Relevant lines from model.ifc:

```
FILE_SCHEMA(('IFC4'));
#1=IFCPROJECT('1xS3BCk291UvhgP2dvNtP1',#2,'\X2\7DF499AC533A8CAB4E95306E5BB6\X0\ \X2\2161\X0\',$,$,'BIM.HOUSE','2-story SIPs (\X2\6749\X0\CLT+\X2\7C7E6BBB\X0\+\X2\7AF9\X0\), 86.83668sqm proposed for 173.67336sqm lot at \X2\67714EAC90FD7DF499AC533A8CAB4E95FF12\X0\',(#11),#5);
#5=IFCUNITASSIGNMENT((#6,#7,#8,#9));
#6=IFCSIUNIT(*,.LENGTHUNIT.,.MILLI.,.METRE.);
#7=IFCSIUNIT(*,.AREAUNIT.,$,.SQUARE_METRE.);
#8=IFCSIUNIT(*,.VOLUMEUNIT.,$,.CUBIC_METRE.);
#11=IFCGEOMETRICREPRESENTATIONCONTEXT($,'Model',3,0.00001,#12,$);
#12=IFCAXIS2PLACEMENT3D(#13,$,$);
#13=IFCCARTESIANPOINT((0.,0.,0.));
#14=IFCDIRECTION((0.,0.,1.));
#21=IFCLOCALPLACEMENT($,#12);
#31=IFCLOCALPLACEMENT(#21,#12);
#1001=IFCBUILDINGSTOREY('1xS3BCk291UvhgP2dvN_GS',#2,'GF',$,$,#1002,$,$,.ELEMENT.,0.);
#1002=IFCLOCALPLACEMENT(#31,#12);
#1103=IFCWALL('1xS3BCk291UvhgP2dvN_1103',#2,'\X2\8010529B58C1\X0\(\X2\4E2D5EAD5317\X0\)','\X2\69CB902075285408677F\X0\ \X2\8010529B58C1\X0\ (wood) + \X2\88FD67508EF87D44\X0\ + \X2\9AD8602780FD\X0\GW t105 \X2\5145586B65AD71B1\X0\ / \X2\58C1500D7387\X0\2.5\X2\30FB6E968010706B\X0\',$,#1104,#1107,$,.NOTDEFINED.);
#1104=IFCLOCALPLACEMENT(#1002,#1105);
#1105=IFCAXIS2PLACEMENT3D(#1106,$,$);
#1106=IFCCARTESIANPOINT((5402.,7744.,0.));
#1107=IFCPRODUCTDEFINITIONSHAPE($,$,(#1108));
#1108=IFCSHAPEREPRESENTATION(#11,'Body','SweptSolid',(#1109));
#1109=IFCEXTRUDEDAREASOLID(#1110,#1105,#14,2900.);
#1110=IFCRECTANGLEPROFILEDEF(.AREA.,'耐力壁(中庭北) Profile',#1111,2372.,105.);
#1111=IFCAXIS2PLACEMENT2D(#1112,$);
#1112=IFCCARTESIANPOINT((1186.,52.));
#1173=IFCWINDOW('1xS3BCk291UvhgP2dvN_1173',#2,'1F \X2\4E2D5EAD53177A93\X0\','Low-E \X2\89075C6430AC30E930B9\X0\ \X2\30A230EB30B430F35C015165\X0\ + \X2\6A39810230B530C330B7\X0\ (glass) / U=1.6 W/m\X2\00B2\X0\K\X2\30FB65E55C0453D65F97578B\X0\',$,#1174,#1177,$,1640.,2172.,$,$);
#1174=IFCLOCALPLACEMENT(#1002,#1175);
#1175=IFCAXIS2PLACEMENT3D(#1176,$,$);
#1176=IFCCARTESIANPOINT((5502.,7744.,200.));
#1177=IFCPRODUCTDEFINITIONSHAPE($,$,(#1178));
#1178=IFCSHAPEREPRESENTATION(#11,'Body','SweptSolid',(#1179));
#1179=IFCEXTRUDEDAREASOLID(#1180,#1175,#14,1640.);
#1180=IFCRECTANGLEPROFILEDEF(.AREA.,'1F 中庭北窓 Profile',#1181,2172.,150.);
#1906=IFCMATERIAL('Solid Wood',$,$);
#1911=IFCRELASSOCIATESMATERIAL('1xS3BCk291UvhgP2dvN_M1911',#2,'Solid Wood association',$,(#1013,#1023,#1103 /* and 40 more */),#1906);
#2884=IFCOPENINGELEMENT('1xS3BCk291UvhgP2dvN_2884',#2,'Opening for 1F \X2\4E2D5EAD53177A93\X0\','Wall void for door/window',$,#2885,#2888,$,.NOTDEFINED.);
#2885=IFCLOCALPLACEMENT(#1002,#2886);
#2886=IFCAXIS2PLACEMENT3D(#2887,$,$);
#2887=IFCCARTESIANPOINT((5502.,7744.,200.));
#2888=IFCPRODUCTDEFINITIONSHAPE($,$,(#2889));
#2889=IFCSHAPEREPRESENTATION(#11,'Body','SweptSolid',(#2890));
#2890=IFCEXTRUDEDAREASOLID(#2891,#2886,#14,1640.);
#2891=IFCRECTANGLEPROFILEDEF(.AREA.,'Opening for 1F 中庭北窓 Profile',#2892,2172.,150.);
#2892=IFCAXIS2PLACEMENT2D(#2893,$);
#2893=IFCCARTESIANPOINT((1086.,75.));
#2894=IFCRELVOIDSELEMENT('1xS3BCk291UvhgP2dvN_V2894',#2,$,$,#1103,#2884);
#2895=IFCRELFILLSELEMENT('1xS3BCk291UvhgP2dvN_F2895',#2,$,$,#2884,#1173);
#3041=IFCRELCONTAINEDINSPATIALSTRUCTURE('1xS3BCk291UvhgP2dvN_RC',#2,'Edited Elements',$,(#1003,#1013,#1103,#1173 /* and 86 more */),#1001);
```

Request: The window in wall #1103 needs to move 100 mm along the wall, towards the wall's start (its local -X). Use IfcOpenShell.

```python
import ifcopenshell
import ifcopenshell.api.geometry
import ifcopenshell.util.placement

model = ifcopenshell.open("model.ifc")

window = model.by_guid("1xS3BCk291UvhgP2dvN_1173")
opening = window.FillsVoids[0].RelatingOpeningElement
wall = opening.VoidsElements[0].RelatingBuildingElement

wall_matrix = ifcopenshell.util.placement.get_local_placement(wall.ObjectPlacement)
shift = wall_matrix[:3, 0] * -100.0
before = ifcopenshell.util.placement.get_local_placement(window.ObjectPlacement)[:3, 3].copy()

# The window is not placed relative to its opening, so move both.
for product in (opening, window):
    matrix = ifcopenshell.util.placement.get_local_placement(product.ObjectPlacement)
    matrix[:3, 3] += shift
    ifcopenshell.api.geometry.edit_object_placement(model, product=product, matrix=matrix, is_si=False)

after = ifcopenshell.util.placement.get_local_placement(window.ObjectPlacement)[:3, 3]
print("window moved by", (after - before).round(3) + 0.0)

model.write("model-out.ifc")
```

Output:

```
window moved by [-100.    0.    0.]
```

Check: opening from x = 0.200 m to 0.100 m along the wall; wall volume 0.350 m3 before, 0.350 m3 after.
